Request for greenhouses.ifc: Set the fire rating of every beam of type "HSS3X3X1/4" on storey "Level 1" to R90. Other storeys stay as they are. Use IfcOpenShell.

First a look at what the model holds.

```python
import ifcopenshell
import ifcopenshell.util.element

model = ifcopenshell.open("greenhouses.ifc")
print(model.schema)
storey = next(s for s in model.by_type("IfcBuildingStorey") if s.Name == "Level 1")
beams = [e for e in ifcopenshell.util.element.get_decomposition(storey) if e.is_a("IfcBeam")]
seen = {}
for e in beams:
    element_type = ifcopenshell.util.element.get_type(e)
    key = (element_type.Name if element_type != e and element_type else None, ifcopenshell.util.element.get_pset(e, "Pset_BeamCommon", "FireRating"))
    seen[key] = seen.get(key, 0) + 1
for (name, value), count in sorted(seen.items(), key=str):
    print(count, "x", name, "|", value)
```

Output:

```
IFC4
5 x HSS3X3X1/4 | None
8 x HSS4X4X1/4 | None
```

```python
import ifcopenshell
import ifcopenshell.api.pset
import ifcopenshell.util.element

model = ifcopenshell.open("greenhouses.ifc")

storey = next(s for s in model.by_type("IfcBuildingStorey") if s.Name == "Level 1")
beams = [e for e in ifcopenshell.util.element.get_decomposition(storey) if e.is_a("IfcBeam")]

count = 0
for e in beams:
    element_type = ifcopenshell.util.element.get_type(e)
    if element_type in (None, e) or element_type.Name != "HSS3X3X1/4":
        continue
    # add_pset returns the element's existing set when there is one.
    pset = ifcopenshell.api.pset.add_pset(model, product=e, name="Pset_BeamCommon")
    ifcopenshell.api.pset.edit_pset(model, pset=pset, properties={"FireRating": "R90"})
    count += 1

print(count, "beams updated")

model.write("greenhouses-out.ifc")
```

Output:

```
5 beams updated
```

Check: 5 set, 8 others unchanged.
